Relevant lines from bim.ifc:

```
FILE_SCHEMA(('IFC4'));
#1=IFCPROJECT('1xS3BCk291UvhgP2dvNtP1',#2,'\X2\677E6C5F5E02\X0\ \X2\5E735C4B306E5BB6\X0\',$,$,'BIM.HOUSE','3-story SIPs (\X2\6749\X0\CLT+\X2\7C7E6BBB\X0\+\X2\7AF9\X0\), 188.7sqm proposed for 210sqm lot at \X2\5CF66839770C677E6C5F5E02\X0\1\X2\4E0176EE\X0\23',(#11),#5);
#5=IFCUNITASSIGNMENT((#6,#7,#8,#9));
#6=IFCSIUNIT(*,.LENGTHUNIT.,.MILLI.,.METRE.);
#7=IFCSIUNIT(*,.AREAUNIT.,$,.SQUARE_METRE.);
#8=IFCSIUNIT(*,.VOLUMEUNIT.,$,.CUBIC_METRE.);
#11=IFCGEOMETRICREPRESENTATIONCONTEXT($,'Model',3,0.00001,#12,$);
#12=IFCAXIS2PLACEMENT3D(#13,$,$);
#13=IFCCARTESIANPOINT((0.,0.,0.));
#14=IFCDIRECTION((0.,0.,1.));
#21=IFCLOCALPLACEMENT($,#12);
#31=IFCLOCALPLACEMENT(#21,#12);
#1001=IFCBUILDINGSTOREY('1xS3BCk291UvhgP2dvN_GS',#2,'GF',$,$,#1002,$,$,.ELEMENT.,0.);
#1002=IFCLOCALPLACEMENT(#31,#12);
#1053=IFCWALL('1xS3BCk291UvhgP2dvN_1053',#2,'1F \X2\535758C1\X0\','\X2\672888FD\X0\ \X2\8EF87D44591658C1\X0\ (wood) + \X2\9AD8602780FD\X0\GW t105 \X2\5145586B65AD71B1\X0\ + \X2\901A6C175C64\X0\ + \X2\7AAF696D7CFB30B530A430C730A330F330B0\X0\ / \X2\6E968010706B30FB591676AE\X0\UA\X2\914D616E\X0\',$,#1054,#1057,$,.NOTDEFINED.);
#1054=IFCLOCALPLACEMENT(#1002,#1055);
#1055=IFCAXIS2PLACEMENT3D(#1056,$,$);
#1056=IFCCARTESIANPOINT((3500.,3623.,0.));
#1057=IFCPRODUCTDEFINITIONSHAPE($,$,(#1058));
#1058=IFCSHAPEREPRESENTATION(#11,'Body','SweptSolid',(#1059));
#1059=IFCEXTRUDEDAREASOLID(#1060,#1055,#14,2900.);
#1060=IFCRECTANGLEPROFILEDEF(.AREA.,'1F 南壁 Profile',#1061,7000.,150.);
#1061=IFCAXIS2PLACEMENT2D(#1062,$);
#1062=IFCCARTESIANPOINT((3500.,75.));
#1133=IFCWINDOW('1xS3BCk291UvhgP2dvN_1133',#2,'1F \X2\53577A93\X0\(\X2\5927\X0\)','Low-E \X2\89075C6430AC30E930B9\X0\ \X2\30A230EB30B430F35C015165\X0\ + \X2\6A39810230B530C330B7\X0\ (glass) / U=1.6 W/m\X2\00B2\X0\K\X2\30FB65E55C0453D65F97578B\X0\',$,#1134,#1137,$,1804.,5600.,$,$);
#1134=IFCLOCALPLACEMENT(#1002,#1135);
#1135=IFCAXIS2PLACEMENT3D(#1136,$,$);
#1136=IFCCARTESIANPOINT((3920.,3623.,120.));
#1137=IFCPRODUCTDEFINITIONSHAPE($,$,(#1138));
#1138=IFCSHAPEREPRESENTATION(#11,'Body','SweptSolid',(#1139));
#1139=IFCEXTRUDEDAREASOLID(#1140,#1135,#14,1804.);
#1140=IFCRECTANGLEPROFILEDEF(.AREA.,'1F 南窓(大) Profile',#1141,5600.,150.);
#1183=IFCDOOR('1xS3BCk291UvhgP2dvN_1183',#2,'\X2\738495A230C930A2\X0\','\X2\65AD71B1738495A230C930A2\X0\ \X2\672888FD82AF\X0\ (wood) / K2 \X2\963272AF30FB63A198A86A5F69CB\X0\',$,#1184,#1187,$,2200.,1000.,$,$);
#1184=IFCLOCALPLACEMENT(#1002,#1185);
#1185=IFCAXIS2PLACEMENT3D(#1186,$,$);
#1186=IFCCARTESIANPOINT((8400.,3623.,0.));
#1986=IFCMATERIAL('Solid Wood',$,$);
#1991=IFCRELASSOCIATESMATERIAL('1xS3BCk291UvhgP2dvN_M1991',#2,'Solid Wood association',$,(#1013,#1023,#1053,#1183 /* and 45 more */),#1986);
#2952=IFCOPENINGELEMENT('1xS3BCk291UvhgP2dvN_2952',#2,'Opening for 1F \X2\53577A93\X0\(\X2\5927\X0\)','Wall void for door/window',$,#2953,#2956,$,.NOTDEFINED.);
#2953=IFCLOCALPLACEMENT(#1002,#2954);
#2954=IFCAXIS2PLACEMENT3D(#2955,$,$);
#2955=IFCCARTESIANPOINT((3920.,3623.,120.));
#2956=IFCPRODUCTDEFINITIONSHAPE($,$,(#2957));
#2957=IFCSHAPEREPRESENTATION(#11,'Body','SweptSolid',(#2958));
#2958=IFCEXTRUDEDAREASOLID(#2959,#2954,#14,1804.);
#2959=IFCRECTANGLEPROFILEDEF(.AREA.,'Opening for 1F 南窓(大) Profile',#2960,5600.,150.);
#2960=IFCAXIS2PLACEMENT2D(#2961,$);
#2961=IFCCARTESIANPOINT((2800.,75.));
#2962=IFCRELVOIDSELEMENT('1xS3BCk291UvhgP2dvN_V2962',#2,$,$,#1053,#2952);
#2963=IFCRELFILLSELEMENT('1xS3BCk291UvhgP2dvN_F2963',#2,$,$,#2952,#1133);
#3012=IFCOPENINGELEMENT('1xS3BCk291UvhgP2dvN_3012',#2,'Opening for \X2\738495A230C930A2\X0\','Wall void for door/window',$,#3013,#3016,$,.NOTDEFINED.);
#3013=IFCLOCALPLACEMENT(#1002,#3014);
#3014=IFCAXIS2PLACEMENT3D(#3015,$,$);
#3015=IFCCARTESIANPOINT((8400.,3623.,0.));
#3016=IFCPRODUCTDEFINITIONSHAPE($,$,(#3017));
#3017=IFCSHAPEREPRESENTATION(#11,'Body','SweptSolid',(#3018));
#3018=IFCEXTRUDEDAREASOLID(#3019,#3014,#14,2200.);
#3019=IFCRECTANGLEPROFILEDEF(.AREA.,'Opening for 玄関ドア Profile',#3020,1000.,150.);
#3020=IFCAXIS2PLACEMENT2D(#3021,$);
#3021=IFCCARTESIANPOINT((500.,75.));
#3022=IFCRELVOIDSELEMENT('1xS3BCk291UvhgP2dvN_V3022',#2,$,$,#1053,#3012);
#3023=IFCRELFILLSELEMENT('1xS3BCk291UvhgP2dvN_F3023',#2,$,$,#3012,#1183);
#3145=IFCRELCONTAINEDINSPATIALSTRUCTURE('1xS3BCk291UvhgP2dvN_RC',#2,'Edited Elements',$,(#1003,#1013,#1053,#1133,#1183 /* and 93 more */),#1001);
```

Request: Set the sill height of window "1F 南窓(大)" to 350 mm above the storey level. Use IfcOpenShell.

```python
import numpy as np
import ifcopenshell
import ifcopenshell.api.geometry
import ifcopenshell.geom
import ifcopenshell.util.element
import ifcopenshell.util.placement
import ifcopenshell.util.shape
import ifcopenshell.util.unit

model = ifcopenshell.open("bim.ifc")
unit_scale = ifcopenshell.util.unit.calculate_unit_scale(model)

window = model.by_guid("1xS3BCk291UvhgP2dvN_1133")
opening = window.FillsVoids[0].RelatingOpeningElement
storey = ifcopenshell.util.element.get_container(window, ifc_class="IfcBuildingStorey")
level = ifcopenshell.util.placement.get_local_placement(storey.ObjectPlacement)[2, 3]

# The opening's origin need not be at the sill, so measure its lowest point.
shape = ifcopenshell.geom.create_shape(ifcopenshell.geom.settings(), opening)
bottom = ifcopenshell.util.shape.get_shape_bottom_elevation(shape, shape.geometry) / unit_scale
dz = level + 0.35 / unit_scale - bottom

shift = np.array([0.0, 0.0, dz])
# The window is not placed relative to its opening, so move both.
for product in (opening, window):
    matrix = ifcopenshell.util.placement.get_local_placement(product.ObjectPlacement)
    matrix[:3, 3] += shift
    ifcopenshell.api.geometry.edit_object_placement(model, product=product, matrix=matrix, is_si=False)

print(f"moved by {dz * unit_scale:+.3f} m")

model.write("bim_rev.ifc")
```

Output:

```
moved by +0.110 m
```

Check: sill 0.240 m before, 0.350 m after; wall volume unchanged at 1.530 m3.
